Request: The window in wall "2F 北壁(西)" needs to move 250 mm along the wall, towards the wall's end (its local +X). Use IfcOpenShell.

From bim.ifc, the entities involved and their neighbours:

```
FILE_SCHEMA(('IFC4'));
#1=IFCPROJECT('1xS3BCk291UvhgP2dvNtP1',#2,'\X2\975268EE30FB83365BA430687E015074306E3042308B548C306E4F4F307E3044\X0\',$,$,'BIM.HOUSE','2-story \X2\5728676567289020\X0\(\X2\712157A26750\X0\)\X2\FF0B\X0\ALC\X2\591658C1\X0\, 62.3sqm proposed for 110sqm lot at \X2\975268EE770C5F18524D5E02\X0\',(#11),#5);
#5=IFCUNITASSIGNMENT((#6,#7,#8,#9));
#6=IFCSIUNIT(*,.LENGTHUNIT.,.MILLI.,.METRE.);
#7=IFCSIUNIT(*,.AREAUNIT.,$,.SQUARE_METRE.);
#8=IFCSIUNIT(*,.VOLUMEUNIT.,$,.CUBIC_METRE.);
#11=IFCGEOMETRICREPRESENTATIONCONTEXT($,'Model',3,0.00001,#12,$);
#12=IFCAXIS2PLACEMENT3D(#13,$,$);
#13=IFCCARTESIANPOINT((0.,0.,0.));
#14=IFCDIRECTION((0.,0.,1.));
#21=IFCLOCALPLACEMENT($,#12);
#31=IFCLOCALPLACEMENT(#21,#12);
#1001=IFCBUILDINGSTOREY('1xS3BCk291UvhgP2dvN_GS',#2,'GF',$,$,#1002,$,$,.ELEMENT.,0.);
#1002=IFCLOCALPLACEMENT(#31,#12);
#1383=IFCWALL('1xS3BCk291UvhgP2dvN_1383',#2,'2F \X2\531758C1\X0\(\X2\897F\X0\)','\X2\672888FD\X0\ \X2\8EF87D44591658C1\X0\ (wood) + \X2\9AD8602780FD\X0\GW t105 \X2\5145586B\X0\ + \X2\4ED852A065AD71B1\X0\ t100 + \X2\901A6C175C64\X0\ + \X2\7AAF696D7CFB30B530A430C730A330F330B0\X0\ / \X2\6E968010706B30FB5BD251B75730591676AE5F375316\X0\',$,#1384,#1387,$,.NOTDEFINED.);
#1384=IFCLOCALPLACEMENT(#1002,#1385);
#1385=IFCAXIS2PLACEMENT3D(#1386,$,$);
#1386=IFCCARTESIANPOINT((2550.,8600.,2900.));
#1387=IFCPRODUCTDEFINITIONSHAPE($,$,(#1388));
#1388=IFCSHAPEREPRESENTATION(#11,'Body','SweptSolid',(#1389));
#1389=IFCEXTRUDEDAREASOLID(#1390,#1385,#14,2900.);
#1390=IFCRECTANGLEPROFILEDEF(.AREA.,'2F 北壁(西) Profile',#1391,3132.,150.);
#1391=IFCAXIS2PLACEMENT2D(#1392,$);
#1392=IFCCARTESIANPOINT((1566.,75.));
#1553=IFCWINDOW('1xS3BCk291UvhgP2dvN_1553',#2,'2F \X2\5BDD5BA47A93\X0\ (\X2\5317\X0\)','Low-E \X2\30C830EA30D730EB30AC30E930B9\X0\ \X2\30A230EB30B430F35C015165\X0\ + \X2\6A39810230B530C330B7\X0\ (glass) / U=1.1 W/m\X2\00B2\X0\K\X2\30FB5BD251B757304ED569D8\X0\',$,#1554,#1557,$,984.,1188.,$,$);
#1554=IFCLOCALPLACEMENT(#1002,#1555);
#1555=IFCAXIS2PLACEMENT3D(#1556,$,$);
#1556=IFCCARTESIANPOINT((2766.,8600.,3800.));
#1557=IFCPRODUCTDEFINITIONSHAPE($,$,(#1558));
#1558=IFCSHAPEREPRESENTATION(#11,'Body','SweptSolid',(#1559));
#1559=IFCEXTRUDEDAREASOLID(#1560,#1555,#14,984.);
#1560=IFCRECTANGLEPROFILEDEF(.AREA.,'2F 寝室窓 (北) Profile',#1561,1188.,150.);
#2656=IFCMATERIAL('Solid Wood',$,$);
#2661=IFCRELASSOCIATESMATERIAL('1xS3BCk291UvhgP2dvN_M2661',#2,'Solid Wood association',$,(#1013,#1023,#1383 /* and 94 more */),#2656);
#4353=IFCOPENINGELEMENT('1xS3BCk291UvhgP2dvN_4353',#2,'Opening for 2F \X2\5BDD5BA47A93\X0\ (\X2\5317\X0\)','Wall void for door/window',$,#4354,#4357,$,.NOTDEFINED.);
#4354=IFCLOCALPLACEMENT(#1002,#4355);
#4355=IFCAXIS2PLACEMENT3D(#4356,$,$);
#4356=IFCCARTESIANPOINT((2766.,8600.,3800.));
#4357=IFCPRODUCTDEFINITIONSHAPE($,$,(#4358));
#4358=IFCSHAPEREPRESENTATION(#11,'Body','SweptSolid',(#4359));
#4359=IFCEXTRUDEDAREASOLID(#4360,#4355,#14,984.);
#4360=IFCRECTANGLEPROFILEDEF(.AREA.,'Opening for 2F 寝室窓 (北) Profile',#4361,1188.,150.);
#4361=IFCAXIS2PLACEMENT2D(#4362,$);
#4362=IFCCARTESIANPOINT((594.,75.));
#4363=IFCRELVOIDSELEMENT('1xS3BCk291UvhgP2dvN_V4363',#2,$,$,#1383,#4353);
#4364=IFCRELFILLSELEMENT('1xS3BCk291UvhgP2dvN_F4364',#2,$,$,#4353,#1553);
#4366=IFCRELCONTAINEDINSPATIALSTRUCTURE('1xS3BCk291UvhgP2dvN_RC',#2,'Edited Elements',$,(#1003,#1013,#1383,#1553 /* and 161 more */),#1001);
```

```python
import ifcopenshell
import ifcopenshell.api.geometry
import ifcopenshell.util.placement

model = ifcopenshell.open("bim.ifc")

window = model.by_id(1553)
opening = window.FillsVoids[0].RelatingOpeningElement
wall = opening.VoidsElements[0].RelatingBuildingElement

wall_matrix = ifcopenshell.util.placement.get_local_placement(wall.ObjectPlacement)
shift = wall_matrix[:3, 0] * 250.0
before = ifcopenshell.util.placement.get_local_placement(window.ObjectPlacement)[:3, 3].copy()

# The window is not placed relative to its opening, so move both.
for product in (opening, window):
    matrix = ifcopenshell.util.placement.get_local_placement(product.ObjectPlacement)
    matrix[:3, 3] += shift
    ifcopenshell.api.geometry.edit_object_placement(model, product=product, matrix=matrix, is_si=False)

after = ifcopenshell.util.placement.get_local_placement(window.ObjectPlacement)[:3, 3]
print("window moved by", (after - before).round(3) + 0.0)

model.write("bim_rev.ifc")
```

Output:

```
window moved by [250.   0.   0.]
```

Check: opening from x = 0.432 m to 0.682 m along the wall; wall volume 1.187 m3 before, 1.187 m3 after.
